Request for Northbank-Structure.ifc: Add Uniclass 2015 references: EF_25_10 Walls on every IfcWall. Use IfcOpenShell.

First a look at what the model holds.

```python
import ifcopenshell

model = ifcopenshell.open("Northbank-Structure.ifc")
print(model.schema)
print("classifications:", [c.Name for c in model.by_type("IfcClassification")])
for ifc_class in ("IfcDoor", "IfcRoof", "IfcStair", "IfcWall", "IfcWindow"):
    print(ifc_class, len(model.by_type(ifc_class)))
```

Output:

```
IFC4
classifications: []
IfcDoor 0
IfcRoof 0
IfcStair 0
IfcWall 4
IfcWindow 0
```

```python
import ifcopenshell
import ifcopenshell.api.classification

model = ifcopenshell.open("Northbank-Structure.ifc")

system = ifcopenshell.api.classification.add_classification(model, classification="Uniclass 2015")

codes = {
    "IfcWall": ("EF_25_10", "Walls"),
}
for ifc_class, (code, name) in codes.items():
    products = model.by_type(ifc_class)
    ifcopenshell.api.classification.add_reference(
        model, products=products, classification=system, identification=code, name=name
    )
    print(code, len(products))

model.write("Northbank-Structure_rev.ifc")
```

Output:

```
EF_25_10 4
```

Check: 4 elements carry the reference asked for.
